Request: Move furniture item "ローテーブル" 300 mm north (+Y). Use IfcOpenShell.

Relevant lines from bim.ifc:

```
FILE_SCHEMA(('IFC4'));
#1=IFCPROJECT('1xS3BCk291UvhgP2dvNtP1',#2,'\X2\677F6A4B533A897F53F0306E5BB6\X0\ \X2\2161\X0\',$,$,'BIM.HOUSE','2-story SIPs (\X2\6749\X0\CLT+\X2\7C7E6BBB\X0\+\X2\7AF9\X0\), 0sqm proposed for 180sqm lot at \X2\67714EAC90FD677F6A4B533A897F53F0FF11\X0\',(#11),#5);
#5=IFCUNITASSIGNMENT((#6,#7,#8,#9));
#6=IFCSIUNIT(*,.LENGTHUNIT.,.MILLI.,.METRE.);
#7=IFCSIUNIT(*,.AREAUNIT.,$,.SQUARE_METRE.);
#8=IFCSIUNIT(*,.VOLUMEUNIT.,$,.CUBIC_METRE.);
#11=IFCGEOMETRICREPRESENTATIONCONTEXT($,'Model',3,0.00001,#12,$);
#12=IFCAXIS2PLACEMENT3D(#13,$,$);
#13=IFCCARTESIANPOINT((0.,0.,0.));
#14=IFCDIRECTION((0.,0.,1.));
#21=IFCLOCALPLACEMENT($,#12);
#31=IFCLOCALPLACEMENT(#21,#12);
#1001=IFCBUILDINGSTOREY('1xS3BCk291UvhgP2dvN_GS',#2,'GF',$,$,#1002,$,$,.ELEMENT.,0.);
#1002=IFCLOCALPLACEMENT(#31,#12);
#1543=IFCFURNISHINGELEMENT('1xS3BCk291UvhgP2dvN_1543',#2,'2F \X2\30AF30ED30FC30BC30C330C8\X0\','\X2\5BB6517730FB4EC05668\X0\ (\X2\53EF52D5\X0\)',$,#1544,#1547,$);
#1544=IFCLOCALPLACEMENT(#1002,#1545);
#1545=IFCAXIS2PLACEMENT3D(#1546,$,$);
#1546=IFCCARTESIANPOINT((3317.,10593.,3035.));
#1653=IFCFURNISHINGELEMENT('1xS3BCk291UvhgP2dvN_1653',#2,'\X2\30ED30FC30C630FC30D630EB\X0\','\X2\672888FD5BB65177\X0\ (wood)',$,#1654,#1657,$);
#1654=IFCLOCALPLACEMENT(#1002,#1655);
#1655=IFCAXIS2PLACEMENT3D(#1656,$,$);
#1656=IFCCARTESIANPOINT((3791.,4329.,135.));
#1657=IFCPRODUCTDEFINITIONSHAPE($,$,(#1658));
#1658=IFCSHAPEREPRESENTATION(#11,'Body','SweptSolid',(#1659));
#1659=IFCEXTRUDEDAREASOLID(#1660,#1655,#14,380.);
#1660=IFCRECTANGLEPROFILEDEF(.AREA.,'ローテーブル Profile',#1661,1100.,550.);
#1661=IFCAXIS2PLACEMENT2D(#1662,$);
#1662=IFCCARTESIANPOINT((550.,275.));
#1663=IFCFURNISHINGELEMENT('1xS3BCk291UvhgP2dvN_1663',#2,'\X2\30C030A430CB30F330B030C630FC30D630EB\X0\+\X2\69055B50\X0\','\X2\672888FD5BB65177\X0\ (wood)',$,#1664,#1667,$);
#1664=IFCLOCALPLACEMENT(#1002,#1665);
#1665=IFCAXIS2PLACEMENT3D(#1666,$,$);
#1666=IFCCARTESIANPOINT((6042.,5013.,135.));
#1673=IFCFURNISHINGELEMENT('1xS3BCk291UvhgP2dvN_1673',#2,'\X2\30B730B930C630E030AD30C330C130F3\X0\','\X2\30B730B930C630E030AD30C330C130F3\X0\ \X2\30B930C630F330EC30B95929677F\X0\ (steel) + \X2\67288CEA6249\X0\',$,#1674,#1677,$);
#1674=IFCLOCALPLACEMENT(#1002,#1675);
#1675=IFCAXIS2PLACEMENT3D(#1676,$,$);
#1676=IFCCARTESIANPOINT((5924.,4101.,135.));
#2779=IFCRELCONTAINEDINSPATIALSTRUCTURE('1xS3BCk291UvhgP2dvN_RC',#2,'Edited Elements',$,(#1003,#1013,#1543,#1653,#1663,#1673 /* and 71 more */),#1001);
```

```python
import ifcopenshell
import ifcopenshell.api.geometry
import ifcopenshell.util.placement
import ifcopenshell.util.unit

model = ifcopenshell.open("bim.ifc")
unit_scale = ifcopenshell.util.unit.calculate_unit_scale(model)

item = model.by_guid("1xS3BCk291UvhgP2dvN_1653")
matrix = ifcopenshell.util.placement.get_local_placement(item.ObjectPlacement)
matrix[1, 3] += 0.3 / unit_scale
ifcopenshell.api.geometry.edit_object_placement(model, product=item, matrix=matrix, is_si=False)

print(ifcopenshell.util.placement.get_local_placement(item.ObjectPlacement).round(3) + 0.0)

model.write("bim_v2.ifc")
```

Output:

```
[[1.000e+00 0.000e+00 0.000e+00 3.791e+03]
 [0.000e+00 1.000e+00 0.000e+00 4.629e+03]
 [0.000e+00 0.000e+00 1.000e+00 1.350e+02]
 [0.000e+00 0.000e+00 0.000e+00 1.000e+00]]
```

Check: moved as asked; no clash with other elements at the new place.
